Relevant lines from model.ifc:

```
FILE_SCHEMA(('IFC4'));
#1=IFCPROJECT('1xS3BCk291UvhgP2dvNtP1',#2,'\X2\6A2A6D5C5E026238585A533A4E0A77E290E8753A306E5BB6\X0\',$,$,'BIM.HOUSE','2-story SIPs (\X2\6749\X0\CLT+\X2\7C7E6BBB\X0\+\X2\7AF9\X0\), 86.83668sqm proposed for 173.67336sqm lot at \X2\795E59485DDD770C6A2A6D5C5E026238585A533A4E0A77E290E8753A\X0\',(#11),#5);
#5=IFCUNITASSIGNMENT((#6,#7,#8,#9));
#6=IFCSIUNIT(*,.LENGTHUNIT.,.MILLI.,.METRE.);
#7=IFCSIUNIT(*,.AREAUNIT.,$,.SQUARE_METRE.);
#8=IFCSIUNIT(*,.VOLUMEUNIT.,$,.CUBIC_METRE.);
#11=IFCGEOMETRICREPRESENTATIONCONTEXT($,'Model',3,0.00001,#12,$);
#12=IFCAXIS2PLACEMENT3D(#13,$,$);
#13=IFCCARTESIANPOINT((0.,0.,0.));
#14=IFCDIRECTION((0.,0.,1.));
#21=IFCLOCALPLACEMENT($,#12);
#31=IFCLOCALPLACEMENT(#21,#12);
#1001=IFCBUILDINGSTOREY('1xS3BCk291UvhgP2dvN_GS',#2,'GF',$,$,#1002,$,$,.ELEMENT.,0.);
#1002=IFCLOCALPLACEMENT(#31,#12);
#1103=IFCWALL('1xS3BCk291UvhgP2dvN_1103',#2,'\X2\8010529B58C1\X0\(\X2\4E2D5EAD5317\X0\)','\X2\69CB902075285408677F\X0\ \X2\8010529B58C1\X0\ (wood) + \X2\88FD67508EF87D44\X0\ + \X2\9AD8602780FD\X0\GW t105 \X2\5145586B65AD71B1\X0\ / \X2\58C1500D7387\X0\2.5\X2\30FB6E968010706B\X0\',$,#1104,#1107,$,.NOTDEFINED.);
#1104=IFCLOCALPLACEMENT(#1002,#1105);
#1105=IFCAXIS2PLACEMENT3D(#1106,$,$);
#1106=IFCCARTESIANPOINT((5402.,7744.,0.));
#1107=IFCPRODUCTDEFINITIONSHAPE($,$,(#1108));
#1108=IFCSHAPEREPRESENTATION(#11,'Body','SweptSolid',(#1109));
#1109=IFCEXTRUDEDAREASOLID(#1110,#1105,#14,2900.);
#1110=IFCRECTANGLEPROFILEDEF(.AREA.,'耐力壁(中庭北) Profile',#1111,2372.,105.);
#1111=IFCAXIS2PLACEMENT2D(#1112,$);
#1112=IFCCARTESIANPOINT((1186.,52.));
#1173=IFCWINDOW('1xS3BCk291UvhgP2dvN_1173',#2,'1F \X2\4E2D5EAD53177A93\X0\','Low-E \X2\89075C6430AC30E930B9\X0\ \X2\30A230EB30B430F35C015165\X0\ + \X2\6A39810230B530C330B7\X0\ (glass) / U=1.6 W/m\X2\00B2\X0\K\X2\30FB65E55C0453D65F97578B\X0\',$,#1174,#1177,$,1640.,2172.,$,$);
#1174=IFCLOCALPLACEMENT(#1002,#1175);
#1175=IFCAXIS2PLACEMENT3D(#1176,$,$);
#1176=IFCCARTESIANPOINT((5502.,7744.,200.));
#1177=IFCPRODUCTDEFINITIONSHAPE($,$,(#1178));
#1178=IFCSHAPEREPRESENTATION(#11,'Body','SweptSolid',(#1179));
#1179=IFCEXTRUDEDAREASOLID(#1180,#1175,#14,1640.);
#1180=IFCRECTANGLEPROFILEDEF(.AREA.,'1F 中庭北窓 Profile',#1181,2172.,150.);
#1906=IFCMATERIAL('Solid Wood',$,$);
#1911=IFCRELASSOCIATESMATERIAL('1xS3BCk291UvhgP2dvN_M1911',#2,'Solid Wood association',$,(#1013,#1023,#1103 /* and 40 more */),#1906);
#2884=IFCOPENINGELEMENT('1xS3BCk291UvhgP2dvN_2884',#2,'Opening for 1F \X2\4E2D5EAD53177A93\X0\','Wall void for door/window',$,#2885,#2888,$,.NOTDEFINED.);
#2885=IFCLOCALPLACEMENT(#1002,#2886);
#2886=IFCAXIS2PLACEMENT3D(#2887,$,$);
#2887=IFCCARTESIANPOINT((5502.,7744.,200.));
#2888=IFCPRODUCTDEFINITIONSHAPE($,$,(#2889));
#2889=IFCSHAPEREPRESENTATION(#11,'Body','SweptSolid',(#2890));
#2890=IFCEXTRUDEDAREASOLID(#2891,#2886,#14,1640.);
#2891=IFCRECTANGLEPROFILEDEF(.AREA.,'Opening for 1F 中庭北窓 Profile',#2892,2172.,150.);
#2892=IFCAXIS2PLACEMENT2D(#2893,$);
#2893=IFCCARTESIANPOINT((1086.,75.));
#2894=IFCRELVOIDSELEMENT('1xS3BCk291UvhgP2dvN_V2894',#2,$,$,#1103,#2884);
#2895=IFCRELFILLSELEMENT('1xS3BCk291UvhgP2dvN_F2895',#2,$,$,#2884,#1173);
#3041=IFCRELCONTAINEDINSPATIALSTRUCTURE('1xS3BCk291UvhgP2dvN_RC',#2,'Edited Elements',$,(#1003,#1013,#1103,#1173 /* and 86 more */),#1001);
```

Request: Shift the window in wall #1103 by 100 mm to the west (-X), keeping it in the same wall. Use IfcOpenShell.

```python
import ifcopenshell
import ifcopenshell.api.geometry
import ifcopenshell.util.placement
import ifcopenshell.util.unit

model = ifcopenshell.open("model.ifc")
unit_scale = ifcopenshell.util.unit.calculate_unit_scale(model)

window = model.by_guid("1xS3BCk291UvhgP2dvN_1173")
opening = window.FillsVoids[0].RelatingOpeningElement
wall = opening.VoidsElements[0].RelatingBuildingElement

wall_matrix = ifcopenshell.util.placement.get_local_placement(wall.ObjectPlacement)
shift = wall_matrix[:3, 0] * -0.1 / unit_scale
before = ifcopenshell.util.placement.get_local_placement(window.ObjectPlacement)[:3, 3].copy()

# The window is not placed relative to its opening, so move both.
for product in (opening, window):
    matrix = ifcopenshell.util.placement.get_local_placement(product.ObjectPlacement)
    matrix[:3, 3] += shift
    ifcopenshell.api.geometry.edit_object_placement(model, product=product, matrix=matrix, is_si=False)

after = ifcopenshell.util.placement.get_local_placement(window.ObjectPlacement)[:3, 3]
print("window moved by", (after - before).round(3) + 0.0)

model.write("model_edited.ifc")
```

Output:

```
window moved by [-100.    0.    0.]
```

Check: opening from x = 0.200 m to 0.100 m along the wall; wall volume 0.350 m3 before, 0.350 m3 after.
